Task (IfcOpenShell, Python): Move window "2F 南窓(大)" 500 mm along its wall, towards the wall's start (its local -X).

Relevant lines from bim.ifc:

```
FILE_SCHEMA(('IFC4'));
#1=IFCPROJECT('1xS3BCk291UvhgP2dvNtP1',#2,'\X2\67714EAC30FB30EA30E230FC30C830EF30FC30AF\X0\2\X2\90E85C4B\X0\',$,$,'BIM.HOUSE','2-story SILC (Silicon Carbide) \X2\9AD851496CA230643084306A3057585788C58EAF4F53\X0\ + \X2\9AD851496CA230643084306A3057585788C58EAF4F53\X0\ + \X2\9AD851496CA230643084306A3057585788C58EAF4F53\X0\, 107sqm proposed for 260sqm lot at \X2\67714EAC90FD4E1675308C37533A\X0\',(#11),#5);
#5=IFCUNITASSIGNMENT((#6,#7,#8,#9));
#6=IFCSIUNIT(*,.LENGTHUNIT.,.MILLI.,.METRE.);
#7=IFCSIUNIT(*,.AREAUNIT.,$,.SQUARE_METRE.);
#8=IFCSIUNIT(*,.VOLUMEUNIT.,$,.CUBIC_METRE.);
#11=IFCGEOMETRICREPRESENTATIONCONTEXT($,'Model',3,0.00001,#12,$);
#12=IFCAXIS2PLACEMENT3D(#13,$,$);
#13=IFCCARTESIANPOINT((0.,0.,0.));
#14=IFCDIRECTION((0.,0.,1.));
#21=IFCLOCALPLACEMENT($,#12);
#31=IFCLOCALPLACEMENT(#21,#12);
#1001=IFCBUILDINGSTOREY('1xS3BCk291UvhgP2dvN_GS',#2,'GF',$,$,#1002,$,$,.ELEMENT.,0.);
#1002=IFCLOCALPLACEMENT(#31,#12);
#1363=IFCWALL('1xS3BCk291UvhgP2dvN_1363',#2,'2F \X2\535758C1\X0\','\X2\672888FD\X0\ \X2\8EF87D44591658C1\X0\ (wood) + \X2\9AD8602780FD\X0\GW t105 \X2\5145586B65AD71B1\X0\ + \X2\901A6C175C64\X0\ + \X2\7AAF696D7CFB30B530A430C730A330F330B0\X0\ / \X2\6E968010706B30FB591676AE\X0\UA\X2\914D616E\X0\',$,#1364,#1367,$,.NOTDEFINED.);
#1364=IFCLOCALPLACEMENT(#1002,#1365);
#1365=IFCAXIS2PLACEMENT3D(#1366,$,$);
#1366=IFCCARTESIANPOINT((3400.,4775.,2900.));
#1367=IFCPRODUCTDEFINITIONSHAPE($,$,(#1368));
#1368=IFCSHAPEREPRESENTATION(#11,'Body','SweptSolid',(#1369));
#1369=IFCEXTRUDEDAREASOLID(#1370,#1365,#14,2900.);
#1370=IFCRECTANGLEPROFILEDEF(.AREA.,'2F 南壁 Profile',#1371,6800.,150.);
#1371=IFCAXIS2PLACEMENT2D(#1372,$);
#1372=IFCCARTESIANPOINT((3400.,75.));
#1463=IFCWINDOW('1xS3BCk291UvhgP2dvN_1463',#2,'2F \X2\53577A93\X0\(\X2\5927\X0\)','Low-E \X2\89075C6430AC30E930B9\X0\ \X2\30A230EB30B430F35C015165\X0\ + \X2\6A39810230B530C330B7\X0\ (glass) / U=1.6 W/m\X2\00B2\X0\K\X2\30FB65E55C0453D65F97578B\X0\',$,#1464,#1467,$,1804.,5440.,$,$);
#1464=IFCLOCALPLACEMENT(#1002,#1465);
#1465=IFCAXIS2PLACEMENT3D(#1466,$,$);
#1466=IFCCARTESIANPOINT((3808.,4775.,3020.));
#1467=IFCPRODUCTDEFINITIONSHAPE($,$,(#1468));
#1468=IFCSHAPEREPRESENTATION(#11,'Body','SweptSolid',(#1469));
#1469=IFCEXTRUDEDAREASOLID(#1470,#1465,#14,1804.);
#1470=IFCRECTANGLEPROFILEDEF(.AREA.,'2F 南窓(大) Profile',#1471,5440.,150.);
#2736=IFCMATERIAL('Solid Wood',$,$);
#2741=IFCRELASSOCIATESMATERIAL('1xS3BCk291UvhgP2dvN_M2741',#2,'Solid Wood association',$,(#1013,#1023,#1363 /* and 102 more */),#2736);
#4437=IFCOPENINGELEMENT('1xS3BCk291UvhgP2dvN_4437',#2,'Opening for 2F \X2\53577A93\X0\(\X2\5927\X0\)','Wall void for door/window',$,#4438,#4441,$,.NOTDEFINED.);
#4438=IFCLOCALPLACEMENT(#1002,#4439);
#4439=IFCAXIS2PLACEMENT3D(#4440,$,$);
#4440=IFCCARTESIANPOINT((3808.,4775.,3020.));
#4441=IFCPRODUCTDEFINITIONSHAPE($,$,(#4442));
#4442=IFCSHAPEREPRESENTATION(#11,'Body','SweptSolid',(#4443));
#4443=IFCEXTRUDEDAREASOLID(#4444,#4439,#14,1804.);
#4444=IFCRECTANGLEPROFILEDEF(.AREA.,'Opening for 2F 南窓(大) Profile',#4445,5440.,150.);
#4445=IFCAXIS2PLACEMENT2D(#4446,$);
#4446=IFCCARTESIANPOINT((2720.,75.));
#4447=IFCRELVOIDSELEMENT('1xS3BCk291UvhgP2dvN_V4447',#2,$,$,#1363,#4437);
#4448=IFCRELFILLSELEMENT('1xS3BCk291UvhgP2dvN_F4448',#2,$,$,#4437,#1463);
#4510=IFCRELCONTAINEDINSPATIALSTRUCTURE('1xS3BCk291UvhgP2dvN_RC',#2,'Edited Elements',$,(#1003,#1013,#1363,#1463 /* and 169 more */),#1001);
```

```python
import ifcopenshell
import ifcopenshell.api.geometry
import ifcopenshell.util.placement

model = ifcopenshell.open("bim.ifc")

window = model.by_guid("1xS3BCk291UvhgP2dvN_1463")
opening = window.FillsVoids[0].RelatingOpeningElement
wall = opening.VoidsElements[0].RelatingBuildingElement

wall_matrix = ifcopenshell.util.placement.get_local_placement(wall.ObjectPlacement)
shift = wall_matrix[:3, 0] * -500.0
before = ifcopenshell.util.placement.get_local_placement(window.ObjectPlacement)[:3, 3].copy()

# The window is not placed relative to its opening, so move both.
for product in (opening, window):
    matrix = ifcopenshell.util.placement.get_local_placement(product.ObjectPlacement)
    matrix[:3, 3] += shift
    ifcopenshell.api.geometry.edit_object_placement(model, product=product, matrix=matrix, is_si=False)

after = ifcopenshell.util.placement.get_local_placement(window.ObjectPlacement)[:3, 3]
print("window moved by", (after - before).round(3) + 0.0)

model.write("bim-out.ifc")
```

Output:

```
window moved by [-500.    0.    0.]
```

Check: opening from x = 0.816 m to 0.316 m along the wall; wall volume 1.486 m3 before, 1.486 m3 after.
